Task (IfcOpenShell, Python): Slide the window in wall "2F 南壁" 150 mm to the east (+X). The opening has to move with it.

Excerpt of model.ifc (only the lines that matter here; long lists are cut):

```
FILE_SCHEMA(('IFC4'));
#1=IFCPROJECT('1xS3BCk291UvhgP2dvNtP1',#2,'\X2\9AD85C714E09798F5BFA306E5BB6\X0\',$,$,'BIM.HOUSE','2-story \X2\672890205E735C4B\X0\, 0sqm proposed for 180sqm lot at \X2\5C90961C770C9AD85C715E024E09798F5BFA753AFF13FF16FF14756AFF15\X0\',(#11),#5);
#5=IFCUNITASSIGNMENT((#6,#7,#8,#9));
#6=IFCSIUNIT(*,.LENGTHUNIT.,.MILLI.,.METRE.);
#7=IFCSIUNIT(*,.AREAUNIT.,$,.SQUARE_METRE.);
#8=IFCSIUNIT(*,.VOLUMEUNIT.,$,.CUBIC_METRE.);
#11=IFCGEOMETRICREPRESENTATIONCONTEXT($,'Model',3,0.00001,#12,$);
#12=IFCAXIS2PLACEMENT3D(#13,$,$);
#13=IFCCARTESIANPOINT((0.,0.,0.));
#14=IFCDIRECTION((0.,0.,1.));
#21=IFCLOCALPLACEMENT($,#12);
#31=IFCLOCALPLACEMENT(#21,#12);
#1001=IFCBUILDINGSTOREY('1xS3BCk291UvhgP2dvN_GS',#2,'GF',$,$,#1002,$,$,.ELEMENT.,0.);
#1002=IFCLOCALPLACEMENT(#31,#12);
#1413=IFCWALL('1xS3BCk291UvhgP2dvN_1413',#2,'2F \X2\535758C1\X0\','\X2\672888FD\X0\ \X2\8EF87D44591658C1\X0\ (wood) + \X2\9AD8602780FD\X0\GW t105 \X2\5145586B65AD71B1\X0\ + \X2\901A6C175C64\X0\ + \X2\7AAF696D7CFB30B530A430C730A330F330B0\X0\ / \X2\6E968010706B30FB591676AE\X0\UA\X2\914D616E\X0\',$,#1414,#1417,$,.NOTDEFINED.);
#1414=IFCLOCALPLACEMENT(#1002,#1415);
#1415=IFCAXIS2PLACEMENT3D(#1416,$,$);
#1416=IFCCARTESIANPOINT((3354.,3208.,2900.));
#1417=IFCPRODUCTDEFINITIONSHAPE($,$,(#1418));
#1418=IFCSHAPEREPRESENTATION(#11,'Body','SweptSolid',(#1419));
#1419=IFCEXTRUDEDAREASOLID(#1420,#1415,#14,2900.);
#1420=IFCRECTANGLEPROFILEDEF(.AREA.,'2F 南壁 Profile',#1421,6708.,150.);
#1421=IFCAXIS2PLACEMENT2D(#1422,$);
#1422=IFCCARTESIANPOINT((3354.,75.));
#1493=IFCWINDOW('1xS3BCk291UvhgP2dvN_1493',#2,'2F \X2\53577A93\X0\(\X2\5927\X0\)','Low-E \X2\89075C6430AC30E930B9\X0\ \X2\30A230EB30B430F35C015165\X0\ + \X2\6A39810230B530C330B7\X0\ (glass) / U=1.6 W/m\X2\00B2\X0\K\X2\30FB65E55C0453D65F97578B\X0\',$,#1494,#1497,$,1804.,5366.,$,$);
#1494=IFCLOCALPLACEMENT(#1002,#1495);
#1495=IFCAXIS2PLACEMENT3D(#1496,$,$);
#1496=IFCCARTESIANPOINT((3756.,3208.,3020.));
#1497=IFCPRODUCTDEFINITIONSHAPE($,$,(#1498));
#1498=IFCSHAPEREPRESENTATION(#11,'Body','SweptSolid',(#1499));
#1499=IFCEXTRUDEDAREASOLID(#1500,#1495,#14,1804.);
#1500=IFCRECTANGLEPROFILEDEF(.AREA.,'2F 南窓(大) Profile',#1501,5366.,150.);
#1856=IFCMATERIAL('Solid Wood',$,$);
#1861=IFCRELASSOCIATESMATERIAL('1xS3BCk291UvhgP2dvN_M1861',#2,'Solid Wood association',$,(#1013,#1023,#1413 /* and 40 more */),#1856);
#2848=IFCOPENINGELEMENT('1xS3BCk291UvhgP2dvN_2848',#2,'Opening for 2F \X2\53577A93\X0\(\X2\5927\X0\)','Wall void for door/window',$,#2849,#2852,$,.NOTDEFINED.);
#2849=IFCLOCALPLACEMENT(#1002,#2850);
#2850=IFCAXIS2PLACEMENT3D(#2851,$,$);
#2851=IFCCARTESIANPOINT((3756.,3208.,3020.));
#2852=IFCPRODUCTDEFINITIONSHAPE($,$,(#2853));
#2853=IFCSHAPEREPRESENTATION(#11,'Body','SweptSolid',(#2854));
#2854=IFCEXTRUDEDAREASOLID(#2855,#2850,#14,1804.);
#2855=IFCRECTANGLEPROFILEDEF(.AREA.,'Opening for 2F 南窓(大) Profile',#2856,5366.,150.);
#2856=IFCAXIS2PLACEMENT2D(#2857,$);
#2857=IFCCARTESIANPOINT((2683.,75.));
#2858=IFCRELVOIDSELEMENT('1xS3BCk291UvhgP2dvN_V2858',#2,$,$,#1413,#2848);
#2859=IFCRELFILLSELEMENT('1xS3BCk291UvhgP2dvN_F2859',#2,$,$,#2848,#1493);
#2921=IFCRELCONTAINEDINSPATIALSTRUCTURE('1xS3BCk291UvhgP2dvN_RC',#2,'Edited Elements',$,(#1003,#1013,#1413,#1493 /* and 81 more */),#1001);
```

```python
import ifcopenshell
import ifcopenshell.api.geometry
import ifcopenshell.util.placement
import ifcopenshell.util.unit

model = ifcopenshell.open("model.ifc")
unit_scale = ifcopenshell.util.unit.calculate_unit_scale(model)

window = model.by_guid("1xS3BCk291UvhgP2dvN_1493")
opening = window.FillsVoids[0].RelatingOpeningElement
wall = opening.VoidsElements[0].RelatingBuildingElement

wall_matrix = ifcopenshell.util.placement.get_local_placement(wall.ObjectPlacement)
shift = wall_matrix[:3, 0] * 0.15 / unit_scale
before = ifcopenshell.util.placement.get_local_placement(window.ObjectPlacement)[:3, 3].copy()

# The window is not placed relative to its opening, so move both.
for product in (opening, window):
    matrix = ifcopenshell.util.placement.get_local_placement(product.ObjectPlacement)
    matrix[:3, 3] += shift
    ifcopenshell.api.geometry.edit_object_placement(model, product=product, matrix=matrix, is_si=False)

after = ifcopenshell.util.placement.get_local_placement(window.ObjectPlacement)[:3, 3]
print("window moved by", (after - before).round(3) + 0.0)

model.write("model_updated.ifc")
```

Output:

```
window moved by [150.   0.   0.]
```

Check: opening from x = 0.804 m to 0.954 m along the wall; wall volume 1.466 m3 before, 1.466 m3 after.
